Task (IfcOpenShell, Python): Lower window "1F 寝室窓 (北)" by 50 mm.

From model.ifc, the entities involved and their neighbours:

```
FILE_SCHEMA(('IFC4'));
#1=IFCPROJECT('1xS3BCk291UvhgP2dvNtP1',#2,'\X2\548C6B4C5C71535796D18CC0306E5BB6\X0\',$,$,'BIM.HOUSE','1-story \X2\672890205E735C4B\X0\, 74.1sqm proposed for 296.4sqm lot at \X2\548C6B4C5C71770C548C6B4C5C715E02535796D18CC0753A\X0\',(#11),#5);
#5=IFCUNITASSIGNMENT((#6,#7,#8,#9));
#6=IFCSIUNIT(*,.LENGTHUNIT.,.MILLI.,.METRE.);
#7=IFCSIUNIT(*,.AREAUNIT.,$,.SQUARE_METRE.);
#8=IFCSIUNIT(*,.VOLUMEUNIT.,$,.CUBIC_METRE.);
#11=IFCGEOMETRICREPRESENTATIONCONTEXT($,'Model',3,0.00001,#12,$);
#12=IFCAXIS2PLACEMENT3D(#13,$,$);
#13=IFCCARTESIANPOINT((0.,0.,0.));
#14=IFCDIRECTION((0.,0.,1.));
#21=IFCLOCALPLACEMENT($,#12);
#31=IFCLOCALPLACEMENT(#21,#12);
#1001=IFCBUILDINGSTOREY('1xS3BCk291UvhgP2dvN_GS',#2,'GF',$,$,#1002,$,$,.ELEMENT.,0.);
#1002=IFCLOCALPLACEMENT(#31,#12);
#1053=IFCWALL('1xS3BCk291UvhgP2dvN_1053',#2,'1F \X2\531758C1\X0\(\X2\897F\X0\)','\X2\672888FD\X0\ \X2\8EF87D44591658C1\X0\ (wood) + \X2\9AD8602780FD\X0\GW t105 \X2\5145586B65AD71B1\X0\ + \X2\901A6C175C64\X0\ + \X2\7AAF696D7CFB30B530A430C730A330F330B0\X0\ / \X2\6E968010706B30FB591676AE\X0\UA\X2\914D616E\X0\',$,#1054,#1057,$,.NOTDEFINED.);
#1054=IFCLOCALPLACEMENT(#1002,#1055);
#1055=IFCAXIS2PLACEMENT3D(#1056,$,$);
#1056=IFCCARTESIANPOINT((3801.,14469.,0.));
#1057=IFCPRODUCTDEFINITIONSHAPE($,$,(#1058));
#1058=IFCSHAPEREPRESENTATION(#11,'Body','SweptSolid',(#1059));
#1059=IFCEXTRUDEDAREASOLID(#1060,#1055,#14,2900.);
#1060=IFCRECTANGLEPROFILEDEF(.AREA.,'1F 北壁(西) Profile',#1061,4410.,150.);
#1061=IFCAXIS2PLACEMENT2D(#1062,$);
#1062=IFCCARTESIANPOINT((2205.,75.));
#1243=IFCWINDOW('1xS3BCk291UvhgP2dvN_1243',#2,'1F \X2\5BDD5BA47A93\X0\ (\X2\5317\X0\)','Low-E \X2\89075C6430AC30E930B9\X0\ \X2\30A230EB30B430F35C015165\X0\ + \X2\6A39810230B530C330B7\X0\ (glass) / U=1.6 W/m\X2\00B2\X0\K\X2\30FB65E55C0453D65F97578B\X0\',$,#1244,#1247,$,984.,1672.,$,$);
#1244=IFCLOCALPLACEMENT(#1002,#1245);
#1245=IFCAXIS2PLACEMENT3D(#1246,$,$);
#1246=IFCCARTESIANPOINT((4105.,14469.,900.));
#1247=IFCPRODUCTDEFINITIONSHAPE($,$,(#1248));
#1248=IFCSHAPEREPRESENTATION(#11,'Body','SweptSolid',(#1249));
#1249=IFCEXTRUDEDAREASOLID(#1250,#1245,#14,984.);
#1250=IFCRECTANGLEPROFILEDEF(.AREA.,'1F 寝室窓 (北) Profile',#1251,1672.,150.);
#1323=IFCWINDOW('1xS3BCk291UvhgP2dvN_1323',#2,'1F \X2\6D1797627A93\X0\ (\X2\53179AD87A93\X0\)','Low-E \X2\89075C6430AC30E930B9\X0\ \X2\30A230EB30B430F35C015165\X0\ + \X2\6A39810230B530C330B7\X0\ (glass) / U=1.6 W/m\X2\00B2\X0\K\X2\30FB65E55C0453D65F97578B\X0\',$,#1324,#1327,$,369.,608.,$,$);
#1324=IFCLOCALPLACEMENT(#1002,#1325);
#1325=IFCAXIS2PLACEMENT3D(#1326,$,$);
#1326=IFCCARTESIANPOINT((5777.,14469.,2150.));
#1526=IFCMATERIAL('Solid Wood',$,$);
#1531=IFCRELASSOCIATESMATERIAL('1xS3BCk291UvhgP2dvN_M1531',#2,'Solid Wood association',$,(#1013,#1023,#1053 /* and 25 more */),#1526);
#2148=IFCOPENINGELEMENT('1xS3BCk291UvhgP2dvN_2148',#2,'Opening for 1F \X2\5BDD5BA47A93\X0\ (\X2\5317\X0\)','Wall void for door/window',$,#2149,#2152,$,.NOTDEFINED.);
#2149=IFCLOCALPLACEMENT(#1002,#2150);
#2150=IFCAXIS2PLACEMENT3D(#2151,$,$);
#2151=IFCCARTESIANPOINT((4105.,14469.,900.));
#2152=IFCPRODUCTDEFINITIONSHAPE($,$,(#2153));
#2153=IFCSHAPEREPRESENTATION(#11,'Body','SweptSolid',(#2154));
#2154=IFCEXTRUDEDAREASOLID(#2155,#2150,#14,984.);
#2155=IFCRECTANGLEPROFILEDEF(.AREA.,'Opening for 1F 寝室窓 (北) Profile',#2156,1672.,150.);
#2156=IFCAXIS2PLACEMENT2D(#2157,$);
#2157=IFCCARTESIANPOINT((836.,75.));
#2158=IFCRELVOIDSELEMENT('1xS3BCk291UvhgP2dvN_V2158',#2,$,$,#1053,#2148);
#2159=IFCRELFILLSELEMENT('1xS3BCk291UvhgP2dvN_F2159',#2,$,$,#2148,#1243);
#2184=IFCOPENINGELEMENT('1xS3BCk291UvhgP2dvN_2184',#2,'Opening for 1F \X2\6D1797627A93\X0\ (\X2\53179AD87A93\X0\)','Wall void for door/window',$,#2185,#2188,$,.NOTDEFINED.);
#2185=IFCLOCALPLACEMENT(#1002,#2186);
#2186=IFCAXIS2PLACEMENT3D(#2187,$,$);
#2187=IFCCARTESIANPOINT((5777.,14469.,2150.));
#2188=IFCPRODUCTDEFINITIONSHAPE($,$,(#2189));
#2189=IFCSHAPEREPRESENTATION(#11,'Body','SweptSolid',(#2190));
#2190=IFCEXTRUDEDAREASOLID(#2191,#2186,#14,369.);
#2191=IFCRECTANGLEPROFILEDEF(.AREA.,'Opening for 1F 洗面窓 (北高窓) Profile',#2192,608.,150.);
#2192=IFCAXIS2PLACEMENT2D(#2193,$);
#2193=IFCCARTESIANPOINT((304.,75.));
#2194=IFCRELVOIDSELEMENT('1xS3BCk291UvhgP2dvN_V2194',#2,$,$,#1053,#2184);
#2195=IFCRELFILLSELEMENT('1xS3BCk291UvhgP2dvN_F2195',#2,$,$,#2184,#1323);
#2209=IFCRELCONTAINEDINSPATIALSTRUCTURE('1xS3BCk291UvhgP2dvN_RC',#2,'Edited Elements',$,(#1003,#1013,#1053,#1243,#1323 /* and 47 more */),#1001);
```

```python
import numpy as np
import ifcopenshell
import ifcopenshell.api.geometry
import ifcopenshell.util.placement
import ifcopenshell.util.unit

model = ifcopenshell.open("model.ifc")
unit_scale = ifcopenshell.util.unit.calculate_unit_scale(model)

window = model.by_guid("1xS3BCk291UvhgP2dvN_1243")
opening = window.FillsVoids[0].RelatingOpeningElement
dz = -0.05 / unit_scale

shift = np.array([0.0, 0.0, dz])
# The window is not placed relative to its opening, so move both.
for product in (opening, window):
    matrix = ifcopenshell.util.placement.get_local_placement(product.ObjectPlacement)
    matrix[:3, 3] += shift
    ifcopenshell.api.geometry.edit_object_placement(model, product=product, matrix=matrix, is_si=False)

print(f"moved by {dz * unit_scale:+.3f} m")

model.write("model-out.ifc")
```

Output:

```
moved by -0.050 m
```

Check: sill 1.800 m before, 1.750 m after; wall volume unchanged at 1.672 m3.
